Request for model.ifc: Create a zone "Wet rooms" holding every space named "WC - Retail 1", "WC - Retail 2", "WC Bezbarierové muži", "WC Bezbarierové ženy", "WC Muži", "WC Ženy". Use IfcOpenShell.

First a look at what the model holds.

```python
import ifcopenshell

model = ifcopenshell.open("model.ifc")
print(model.schema)
seen = {}
for space in model.by_type("IfcSpace"):
    seen[space.LongName] = seen.get(space.LongName, 0) + 1
for name, count in sorted(seen.items(), key=str):
    print(count, "x", name)
print("zones:", [z.Name for z in model.by_type("IfcZone")][:20])
```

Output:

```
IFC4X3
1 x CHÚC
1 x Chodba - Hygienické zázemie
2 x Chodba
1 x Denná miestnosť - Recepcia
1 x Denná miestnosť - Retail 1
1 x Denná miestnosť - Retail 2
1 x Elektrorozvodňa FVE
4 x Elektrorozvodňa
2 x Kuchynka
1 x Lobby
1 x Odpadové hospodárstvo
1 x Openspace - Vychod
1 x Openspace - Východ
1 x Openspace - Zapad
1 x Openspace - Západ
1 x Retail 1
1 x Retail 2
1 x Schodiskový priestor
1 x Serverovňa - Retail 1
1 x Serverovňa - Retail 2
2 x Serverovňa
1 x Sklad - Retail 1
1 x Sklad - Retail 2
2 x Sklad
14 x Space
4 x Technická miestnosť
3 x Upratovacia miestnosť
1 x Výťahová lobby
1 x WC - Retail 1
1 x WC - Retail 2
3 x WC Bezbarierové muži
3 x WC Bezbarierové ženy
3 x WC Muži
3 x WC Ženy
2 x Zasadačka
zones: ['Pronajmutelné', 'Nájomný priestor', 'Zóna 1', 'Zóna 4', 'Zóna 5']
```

```python
import ifcopenshell
import ifcopenshell.api.group
import ifcopenshell.api.root

model = ifcopenshell.open("model.ifc")

names = {"WC - Retail 1", "WC - Retail 2", "WC Bezbarierové muži", "WC Bezbarierové ženy", "WC Muži", "WC Ženy"}
spaces = [s for s in model.by_type("IfcSpace") if s.LongName in names]

zone = ifcopenshell.api.root.create_entity(model, ifc_class="IfcZone", name="Wet rooms")
ifcopenshell.api.group.assign_group(model, products=spaces, group=zone)
print(len(spaces), "spaces in", zone.Name)

model.write("model-out.ifc")
```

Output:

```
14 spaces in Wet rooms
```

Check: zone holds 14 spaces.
